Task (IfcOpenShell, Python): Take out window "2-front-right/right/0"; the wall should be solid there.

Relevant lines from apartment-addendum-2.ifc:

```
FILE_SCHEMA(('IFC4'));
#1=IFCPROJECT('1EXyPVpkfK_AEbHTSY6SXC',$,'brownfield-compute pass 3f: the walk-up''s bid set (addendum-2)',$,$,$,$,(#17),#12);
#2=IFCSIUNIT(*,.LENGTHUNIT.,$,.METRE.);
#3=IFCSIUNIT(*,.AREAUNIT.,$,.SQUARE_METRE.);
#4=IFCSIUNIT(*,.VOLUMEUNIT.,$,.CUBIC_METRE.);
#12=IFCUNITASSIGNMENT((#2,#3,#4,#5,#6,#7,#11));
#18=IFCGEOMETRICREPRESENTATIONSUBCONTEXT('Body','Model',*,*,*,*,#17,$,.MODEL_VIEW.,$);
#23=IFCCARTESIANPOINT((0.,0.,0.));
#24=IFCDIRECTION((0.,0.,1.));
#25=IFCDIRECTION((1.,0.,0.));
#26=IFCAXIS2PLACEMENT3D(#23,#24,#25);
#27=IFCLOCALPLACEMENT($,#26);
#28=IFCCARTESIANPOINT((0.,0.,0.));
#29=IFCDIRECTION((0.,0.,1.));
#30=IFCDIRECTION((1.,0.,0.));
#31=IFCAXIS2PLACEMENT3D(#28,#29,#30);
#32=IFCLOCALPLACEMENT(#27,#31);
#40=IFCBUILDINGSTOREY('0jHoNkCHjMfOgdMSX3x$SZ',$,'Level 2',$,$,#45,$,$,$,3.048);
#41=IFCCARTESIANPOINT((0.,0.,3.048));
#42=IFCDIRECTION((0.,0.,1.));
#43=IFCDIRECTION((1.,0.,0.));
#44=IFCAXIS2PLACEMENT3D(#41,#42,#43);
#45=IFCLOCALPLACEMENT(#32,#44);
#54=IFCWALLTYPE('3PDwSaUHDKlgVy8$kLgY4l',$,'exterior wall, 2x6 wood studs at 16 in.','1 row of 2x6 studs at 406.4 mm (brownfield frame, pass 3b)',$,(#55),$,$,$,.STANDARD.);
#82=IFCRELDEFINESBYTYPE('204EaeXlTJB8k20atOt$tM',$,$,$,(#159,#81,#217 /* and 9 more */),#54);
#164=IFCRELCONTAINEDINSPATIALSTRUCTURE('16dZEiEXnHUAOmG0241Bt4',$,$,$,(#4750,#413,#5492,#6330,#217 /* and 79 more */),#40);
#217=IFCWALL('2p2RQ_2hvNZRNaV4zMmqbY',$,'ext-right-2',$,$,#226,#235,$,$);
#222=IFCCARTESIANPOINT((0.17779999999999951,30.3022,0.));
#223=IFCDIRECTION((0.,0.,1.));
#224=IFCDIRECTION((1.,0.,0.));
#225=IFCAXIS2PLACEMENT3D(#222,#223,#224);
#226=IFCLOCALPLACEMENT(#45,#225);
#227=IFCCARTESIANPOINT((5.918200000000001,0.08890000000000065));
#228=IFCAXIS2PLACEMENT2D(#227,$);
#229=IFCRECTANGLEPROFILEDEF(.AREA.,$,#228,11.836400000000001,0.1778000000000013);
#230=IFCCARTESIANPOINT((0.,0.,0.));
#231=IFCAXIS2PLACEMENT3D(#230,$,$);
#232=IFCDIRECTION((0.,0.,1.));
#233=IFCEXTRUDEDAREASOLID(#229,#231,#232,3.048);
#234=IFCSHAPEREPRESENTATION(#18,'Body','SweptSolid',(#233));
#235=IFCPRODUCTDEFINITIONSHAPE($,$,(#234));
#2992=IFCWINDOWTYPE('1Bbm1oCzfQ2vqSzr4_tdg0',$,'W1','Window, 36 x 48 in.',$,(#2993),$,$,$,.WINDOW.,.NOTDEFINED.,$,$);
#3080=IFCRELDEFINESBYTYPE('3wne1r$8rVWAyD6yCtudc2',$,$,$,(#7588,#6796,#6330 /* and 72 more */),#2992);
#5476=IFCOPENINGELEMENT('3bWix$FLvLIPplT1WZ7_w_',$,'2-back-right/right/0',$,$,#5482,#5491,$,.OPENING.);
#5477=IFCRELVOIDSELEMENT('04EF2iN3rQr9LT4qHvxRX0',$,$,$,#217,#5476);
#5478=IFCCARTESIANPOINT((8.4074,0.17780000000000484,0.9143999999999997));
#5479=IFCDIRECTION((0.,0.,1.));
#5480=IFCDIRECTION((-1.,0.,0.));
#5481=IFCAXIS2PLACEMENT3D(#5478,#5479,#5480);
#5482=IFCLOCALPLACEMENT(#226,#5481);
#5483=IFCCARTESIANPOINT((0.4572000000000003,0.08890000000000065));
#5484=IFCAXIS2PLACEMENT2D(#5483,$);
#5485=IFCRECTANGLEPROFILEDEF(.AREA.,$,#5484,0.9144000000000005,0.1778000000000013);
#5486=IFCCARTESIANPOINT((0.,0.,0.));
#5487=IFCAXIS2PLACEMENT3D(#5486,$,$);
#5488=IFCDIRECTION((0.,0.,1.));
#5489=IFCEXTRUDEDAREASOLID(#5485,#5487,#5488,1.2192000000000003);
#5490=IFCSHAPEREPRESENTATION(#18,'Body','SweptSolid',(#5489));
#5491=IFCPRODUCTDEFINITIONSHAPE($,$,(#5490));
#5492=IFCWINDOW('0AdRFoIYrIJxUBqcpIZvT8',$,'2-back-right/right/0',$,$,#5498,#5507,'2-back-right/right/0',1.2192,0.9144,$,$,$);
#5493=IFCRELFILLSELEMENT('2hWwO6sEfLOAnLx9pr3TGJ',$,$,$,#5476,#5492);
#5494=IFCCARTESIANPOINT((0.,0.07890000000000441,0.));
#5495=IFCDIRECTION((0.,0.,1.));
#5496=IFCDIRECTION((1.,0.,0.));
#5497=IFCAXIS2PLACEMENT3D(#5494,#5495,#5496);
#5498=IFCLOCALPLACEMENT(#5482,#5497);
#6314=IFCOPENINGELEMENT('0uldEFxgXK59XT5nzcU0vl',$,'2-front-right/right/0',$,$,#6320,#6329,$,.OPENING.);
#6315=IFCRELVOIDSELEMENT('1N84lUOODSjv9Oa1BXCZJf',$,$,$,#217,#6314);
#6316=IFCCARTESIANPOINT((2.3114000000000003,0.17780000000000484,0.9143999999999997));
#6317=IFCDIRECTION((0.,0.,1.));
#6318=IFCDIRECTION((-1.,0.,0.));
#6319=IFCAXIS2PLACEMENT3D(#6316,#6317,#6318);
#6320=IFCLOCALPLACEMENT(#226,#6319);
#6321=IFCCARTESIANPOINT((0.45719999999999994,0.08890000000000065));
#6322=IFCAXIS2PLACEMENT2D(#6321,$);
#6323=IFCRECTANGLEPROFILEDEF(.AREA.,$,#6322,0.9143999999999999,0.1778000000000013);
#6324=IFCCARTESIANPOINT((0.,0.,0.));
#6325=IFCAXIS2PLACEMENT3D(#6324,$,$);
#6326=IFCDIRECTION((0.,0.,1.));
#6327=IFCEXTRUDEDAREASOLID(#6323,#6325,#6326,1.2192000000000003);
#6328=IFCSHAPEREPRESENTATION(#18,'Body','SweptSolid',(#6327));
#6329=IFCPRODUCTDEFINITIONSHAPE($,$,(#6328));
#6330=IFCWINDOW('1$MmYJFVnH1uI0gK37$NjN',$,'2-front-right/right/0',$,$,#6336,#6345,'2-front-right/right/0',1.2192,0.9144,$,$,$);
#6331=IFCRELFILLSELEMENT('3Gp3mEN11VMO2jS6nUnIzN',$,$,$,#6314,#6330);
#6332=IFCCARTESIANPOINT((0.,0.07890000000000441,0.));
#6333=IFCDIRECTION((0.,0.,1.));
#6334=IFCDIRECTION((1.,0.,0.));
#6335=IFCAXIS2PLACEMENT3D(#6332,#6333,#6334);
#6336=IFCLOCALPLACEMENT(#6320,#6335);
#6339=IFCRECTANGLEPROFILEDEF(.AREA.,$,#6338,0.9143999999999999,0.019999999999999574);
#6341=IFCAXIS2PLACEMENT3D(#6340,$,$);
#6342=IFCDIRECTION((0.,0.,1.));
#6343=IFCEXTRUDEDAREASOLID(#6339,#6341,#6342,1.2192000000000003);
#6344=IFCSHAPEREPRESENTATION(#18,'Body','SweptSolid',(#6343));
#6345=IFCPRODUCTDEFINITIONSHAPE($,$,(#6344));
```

```python
import ifcopenshell
import ifcopenshell.api.feature
import ifcopenshell.api.root
import ifcopenshell.geom
import ifcopenshell.util.shape

model = ifcopenshell.open("apartment-addendum-2.ifc")
settings = ifcopenshell.geom.settings()


def volume(element):
    """Net volume in cubic metres, openings subtracted."""
    shape = ifcopenshell.geom.create_shape(settings, element)
    return ifcopenshell.util.shape.get_volume(shape.geometry)


window = model.by_id(6330)
opening = window.FillsVoids[0].RelatingOpeningElement
wall = opening.VoidsElements[0].RelatingBuildingElement
before = volume(wall)

ifcopenshell.api.root.remove_product(model, product=window)
ifcopenshell.api.feature.remove_feature(model, feature=opening)

after = volume(wall)

print(f"wall volume {before:.3f} -> {after:.3f} m3")

model.write("apartment-addendum-2_rev.ifc")
```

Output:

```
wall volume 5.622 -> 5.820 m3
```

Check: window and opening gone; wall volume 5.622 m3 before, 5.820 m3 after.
